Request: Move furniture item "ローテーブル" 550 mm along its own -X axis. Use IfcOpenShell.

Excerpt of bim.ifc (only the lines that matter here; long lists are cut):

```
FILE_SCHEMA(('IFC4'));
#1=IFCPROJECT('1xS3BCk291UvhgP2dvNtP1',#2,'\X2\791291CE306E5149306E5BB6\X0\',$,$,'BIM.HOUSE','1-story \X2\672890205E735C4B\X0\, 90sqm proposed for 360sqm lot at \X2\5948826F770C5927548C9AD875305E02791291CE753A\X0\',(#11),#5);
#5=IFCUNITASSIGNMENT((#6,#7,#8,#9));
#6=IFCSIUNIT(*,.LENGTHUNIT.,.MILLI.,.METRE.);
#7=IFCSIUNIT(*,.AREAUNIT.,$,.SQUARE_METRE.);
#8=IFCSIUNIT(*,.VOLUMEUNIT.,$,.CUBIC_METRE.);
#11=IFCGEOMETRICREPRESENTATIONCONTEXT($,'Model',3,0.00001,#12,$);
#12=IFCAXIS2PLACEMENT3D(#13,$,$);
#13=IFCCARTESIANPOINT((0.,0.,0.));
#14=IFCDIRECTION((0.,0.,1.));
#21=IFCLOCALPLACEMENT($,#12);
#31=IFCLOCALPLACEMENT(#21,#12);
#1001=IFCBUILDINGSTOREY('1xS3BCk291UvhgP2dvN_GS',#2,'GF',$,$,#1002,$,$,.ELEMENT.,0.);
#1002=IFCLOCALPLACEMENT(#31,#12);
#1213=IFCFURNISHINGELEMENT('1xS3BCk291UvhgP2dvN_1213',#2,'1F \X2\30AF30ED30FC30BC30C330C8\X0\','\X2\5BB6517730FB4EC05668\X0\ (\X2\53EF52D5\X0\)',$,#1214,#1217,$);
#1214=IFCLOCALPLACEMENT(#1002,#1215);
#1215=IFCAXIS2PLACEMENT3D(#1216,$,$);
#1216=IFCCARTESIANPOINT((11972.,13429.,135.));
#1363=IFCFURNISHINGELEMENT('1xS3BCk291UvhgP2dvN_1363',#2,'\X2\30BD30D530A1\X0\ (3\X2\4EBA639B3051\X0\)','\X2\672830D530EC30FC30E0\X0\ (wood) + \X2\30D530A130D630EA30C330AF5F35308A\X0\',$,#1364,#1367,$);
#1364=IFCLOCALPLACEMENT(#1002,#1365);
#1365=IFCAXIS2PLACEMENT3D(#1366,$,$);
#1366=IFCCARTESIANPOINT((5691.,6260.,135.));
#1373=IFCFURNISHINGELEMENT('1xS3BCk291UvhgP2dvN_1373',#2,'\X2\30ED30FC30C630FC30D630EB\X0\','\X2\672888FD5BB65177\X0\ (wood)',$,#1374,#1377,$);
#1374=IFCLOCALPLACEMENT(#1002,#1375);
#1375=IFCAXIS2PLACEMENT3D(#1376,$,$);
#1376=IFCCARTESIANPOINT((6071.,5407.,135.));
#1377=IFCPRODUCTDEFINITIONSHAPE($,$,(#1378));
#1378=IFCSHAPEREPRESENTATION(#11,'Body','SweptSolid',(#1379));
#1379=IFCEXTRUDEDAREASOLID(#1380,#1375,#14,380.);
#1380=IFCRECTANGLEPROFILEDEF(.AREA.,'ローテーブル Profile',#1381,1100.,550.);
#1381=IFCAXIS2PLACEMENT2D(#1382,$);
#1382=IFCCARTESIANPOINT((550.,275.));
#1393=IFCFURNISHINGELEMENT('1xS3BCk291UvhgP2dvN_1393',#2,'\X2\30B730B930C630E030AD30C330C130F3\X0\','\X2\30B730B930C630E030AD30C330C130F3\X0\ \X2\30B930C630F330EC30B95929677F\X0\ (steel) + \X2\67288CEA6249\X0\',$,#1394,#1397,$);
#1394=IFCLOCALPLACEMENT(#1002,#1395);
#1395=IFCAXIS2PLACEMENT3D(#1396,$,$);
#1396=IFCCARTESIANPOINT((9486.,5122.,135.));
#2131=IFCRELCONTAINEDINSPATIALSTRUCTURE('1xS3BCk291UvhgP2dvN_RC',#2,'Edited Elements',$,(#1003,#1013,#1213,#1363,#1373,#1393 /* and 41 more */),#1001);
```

```python
import ifcopenshell
import ifcopenshell.api.geometry
import ifcopenshell.util.placement
import ifcopenshell.util.unit

model = ifcopenshell.open("bim.ifc")
unit_scale = ifcopenshell.util.unit.calculate_unit_scale(model)

item = model.by_guid("1xS3BCk291UvhgP2dvN_1373")
matrix = ifcopenshell.util.placement.get_local_placement(item.ObjectPlacement)
matrix[:3, 3] -= matrix[:3, 0] * 0.55 / unit_scale
ifcopenshell.api.geometry.edit_object_placement(model, product=item, matrix=matrix, is_si=False)

print(ifcopenshell.util.placement.get_local_placement(item.ObjectPlacement).round(3) + 0.0)

model.write("bim_edited.ifc")
```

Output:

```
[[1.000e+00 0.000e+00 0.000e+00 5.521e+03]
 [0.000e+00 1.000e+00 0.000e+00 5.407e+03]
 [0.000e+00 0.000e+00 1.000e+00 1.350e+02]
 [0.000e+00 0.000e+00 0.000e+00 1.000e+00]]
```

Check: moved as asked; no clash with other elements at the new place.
